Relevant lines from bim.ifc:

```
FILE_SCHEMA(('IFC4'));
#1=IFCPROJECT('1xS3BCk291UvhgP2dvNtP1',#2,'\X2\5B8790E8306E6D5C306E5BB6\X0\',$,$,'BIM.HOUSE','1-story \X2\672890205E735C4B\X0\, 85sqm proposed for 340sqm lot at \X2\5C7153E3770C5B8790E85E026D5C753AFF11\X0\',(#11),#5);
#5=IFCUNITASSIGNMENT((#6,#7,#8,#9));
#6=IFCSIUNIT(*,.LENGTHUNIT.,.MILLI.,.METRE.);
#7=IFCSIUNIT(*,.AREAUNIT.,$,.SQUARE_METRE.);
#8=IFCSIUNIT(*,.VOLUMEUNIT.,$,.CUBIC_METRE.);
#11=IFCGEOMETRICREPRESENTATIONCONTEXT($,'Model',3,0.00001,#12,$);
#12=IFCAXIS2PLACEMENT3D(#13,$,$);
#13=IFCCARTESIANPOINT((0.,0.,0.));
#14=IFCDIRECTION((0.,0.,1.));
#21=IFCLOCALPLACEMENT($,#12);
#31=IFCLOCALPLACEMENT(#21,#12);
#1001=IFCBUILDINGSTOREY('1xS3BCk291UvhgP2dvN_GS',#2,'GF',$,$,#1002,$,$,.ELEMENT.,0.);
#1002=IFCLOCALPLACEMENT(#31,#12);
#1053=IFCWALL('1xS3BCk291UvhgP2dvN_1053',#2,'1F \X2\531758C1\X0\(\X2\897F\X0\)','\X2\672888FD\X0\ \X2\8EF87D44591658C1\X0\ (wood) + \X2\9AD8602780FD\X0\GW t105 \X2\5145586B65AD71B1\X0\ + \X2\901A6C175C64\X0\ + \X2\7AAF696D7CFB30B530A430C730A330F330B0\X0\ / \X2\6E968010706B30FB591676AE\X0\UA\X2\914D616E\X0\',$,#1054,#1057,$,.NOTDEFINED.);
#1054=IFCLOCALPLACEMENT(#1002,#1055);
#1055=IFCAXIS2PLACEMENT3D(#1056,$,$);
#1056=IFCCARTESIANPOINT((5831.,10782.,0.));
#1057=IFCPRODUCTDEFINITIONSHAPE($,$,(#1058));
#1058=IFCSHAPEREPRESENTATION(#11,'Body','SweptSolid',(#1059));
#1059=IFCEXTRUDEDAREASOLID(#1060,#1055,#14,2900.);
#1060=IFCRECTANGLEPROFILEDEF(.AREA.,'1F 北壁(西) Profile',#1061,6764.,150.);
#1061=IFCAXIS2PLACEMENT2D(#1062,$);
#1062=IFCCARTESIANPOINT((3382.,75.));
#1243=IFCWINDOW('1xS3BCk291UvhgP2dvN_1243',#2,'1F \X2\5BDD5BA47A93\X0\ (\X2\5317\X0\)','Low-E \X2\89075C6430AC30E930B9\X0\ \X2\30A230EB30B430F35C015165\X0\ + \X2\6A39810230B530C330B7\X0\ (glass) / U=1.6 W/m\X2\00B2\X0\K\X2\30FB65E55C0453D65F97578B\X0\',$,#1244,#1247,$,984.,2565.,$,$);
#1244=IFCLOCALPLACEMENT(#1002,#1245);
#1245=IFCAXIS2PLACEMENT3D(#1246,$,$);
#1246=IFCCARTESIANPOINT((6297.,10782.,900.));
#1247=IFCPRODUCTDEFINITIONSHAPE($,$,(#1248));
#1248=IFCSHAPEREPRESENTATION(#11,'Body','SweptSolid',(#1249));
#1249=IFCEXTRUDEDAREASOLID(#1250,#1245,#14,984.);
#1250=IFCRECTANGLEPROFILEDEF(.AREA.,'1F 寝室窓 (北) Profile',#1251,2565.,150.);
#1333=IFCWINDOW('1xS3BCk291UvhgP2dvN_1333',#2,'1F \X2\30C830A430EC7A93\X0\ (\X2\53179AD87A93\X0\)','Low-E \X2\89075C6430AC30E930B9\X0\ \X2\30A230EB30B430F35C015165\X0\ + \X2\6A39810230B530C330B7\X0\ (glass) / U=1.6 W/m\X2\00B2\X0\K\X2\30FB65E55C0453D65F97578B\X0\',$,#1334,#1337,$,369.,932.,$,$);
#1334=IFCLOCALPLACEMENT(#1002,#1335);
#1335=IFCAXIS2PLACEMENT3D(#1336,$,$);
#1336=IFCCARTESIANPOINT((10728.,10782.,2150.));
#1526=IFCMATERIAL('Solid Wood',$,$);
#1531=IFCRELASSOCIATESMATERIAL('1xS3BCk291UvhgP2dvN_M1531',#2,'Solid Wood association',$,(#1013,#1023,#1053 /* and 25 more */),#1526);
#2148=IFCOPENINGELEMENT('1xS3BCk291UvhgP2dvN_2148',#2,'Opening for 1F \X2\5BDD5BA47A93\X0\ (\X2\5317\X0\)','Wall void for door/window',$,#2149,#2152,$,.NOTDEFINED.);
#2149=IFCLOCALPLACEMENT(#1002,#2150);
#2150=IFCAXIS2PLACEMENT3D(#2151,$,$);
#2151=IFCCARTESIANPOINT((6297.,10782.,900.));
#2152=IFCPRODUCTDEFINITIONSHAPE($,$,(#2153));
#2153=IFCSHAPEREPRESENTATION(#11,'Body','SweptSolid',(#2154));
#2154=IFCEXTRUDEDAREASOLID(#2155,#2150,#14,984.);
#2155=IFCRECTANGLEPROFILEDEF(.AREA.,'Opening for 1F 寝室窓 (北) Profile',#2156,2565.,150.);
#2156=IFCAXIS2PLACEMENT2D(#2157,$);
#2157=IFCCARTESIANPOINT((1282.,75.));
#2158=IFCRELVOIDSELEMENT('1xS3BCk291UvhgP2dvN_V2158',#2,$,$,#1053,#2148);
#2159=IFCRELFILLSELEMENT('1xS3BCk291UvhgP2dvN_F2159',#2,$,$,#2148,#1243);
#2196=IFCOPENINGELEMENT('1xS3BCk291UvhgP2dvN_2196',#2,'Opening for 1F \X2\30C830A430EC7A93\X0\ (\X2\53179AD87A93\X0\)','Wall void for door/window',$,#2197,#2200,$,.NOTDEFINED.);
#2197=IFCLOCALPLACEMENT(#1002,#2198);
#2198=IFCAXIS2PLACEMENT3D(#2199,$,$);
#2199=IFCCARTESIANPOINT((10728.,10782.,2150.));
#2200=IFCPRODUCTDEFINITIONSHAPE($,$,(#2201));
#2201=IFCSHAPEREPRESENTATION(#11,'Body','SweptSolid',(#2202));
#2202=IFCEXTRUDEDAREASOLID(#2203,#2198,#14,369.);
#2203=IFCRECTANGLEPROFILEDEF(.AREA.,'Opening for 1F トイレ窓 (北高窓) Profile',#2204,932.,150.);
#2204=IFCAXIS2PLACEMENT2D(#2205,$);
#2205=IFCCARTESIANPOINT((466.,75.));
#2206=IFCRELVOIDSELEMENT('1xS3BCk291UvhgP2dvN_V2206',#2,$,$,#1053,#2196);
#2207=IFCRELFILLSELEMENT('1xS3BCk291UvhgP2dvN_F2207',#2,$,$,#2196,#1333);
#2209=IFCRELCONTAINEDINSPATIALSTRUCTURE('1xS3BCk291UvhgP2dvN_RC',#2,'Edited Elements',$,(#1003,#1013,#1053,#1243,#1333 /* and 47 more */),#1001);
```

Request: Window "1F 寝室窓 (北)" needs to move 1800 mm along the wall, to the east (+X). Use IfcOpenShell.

```python
import ifcopenshell
import ifcopenshell.api.geometry
import ifcopenshell.util.placement

model = ifcopenshell.open("bim.ifc")

window = model.by_id(1243)
opening = window.FillsVoids[0].RelatingOpeningElement
wall = opening.VoidsElements[0].RelatingBuildingElement

wall_matrix = ifcopenshell.util.placement.get_local_placement(wall.ObjectPlacement)
shift = wall_matrix[:3, 0] * 1800.0
before = ifcopenshell.util.placement.get_local_placement(window.ObjectPlacement)[:3, 3].copy()

# The window is not placed relative to its opening, so move both.
for product in (opening, window):
    matrix = ifcopenshell.util.placement.get_local_placement(product.ObjectPlacement)
    matrix[:3, 3] += shift
    ifcopenshell.api.geometry.edit_object_placement(model, product=product, matrix=matrix, is_si=False)

after = ifcopenshell.util.placement.get_local_placement(window.ObjectPlacement)[:3, 3]
print("window moved by", (after - before).round(3) + 0.0)

model.write("bim_updated.ifc")
```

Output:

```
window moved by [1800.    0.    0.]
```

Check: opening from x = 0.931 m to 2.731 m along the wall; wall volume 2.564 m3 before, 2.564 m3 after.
